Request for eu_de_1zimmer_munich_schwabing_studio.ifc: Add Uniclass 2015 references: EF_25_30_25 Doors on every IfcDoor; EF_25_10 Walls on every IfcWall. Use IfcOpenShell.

First a look at what the model holds.

```python
import ifcopenshell

model = ifcopenshell.open("eu_de_1zimmer_munich_schwabing_studio.ifc")
print(model.schema)
print("classifications:", [c.Name for c in model.by_type("IfcClassification")])
for ifc_class in ("IfcDoor", "IfcRoof", "IfcStair", "IfcWall", "IfcWindow"):
    print(ifc_class, len(model.by_type(ifc_class)))
```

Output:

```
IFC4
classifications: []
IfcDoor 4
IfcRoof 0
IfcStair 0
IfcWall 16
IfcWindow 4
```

```python
import ifcopenshell
import ifcopenshell.api.classification

model = ifcopenshell.open("eu_de_1zimmer_munich_schwabing_studio.ifc")

system = ifcopenshell.api.classification.add_classification(model, classification="Uniclass 2015")

codes = {
    "IfcDoor": ("EF_25_30_25", "Doors"),
    "IfcWall": ("EF_25_10", "Walls"),
}
for ifc_class, (code, name) in codes.items():
    products = model.by_type(ifc_class)
    ifcopenshell.api.classification.add_reference(
        model, products=products, classification=system, identification=code, name=name
    )
    print(code, len(products))

model.write("eu_de_1zimmer_munich_schwabing_studio-out.ifc")
```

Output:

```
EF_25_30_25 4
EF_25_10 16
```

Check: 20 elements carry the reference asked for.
